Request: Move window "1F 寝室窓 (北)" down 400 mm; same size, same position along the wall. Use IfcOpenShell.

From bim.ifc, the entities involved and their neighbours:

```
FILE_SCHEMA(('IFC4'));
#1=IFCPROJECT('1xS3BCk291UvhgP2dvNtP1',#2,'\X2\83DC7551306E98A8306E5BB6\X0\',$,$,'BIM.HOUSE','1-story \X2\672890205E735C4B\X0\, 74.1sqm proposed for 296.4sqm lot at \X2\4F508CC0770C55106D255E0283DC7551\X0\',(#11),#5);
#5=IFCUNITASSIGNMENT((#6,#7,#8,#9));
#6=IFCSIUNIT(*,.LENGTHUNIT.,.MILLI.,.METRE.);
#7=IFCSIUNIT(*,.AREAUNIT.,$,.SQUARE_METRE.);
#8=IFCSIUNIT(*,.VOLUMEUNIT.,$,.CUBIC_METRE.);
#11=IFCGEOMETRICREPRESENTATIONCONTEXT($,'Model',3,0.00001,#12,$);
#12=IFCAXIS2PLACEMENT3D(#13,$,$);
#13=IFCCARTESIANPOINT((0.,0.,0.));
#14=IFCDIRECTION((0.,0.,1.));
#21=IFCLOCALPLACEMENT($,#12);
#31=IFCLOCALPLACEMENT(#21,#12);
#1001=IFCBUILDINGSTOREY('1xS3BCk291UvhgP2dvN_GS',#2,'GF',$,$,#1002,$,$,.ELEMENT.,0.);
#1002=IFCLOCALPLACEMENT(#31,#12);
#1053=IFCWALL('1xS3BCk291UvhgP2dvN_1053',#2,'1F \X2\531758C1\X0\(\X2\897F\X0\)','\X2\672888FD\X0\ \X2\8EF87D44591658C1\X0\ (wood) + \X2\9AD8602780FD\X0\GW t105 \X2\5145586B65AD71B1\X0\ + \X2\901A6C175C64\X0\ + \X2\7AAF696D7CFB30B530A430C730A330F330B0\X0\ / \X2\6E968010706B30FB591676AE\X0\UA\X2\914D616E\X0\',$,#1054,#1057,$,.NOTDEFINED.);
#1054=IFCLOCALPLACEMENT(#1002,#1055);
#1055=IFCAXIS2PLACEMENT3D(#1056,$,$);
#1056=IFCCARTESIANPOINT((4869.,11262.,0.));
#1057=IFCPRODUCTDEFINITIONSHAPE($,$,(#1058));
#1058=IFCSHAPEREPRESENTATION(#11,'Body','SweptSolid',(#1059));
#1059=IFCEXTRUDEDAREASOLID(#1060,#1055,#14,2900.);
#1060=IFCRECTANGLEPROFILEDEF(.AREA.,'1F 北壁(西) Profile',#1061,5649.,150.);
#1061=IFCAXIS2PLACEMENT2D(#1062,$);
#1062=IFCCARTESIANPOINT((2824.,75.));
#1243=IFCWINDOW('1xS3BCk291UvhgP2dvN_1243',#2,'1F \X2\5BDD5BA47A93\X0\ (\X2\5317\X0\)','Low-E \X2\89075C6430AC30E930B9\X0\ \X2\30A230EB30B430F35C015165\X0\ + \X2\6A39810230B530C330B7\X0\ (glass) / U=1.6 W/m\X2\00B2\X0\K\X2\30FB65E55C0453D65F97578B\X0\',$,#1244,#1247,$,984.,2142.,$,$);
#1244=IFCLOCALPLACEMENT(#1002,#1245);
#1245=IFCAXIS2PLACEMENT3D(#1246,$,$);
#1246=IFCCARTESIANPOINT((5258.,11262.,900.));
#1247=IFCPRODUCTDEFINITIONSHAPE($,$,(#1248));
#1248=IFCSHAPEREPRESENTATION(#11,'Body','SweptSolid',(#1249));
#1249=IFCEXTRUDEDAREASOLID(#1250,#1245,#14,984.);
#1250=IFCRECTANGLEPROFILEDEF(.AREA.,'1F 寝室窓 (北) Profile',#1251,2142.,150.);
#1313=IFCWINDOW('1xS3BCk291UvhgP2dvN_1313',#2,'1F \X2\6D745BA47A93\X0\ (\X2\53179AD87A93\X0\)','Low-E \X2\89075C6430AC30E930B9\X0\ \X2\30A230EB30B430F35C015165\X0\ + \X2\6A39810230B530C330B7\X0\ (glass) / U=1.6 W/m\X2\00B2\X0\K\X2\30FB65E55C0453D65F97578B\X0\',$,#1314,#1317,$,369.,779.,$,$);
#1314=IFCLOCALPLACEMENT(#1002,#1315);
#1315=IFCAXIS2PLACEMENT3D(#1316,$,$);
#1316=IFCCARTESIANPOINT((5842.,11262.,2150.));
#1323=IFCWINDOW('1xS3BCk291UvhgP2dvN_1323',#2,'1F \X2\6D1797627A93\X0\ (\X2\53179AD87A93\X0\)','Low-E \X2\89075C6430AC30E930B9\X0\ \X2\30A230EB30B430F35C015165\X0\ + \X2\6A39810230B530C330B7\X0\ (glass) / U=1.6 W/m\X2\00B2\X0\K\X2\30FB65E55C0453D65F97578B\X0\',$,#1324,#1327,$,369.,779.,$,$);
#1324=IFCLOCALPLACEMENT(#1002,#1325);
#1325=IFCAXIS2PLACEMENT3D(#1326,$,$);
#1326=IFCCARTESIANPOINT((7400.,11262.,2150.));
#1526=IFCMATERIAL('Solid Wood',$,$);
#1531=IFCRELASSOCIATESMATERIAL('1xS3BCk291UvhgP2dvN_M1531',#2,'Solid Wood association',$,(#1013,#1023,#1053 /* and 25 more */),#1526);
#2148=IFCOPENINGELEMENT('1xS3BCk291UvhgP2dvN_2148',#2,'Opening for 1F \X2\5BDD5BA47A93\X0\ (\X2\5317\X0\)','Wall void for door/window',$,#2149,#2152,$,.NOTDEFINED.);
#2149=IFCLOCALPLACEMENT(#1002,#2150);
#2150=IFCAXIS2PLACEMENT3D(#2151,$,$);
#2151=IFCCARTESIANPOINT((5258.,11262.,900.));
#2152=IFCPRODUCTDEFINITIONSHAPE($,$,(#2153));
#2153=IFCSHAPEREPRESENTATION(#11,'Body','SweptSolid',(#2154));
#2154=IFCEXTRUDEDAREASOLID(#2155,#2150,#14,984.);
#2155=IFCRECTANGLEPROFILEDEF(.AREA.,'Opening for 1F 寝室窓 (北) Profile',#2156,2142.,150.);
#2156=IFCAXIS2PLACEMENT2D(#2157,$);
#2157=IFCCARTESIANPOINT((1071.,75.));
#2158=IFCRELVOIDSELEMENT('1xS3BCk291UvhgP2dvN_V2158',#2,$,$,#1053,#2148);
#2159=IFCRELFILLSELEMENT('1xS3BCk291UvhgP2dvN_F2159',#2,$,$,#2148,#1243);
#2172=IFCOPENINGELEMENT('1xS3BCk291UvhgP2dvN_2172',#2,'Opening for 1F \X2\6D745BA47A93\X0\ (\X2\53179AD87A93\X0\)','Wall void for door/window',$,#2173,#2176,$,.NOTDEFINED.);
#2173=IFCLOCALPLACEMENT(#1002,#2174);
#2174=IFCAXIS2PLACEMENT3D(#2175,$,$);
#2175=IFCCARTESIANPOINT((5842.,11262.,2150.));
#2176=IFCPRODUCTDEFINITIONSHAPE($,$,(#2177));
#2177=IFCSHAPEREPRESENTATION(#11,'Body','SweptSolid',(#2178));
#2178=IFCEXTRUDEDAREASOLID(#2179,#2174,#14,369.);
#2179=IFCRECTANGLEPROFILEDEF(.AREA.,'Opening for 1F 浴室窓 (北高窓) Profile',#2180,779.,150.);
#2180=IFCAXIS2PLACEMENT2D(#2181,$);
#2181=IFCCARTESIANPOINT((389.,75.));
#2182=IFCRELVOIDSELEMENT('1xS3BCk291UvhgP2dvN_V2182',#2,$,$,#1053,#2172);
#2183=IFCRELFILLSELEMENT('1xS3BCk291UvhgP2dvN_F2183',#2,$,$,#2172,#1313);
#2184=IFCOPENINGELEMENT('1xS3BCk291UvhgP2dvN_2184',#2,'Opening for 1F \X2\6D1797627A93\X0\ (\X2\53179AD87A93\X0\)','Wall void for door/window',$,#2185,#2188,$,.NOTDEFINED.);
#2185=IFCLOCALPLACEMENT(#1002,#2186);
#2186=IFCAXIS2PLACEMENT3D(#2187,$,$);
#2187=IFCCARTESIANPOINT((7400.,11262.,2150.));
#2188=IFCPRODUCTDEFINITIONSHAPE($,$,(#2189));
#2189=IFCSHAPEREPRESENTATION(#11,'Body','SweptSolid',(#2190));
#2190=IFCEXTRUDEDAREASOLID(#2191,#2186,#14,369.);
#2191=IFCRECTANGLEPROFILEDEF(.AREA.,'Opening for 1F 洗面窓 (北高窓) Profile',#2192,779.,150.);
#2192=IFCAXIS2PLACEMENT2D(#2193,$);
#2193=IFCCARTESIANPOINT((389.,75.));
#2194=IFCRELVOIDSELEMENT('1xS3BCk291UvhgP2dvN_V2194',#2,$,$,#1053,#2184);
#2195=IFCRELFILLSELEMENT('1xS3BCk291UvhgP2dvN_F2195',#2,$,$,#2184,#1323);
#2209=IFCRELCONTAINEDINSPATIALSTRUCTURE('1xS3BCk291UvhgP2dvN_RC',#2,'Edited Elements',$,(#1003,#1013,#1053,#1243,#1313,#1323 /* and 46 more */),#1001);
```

```python
import numpy as np
import ifcopenshell
import ifcopenshell.api.geometry
import ifcopenshell.util.placement
import ifcopenshell.util.unit

model = ifcopenshell.open("bim.ifc")
unit_scale = ifcopenshell.util.unit.calculate_unit_scale(model)

window = model.by_id(1243)
opening = window.FillsVoids[0].RelatingOpeningElement
dz = -0.4 / unit_scale

shift = np.array([0.0, 0.0, dz])
# The window is not placed relative to its opening, so move both.
for product in (opening, window):
    matrix = ifcopenshell.util.placement.get_local_placement(product.ObjectPlacement)
    matrix[:3, 3] += shift
    ifcopenshell.api.geometry.edit_object_placement(model, product=product, matrix=matrix, is_si=False)

print(f"moved by {dz * unit_scale:+.3f} m")

model.write("bim_rev.ifc")
```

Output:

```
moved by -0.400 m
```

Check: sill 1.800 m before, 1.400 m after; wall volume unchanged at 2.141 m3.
